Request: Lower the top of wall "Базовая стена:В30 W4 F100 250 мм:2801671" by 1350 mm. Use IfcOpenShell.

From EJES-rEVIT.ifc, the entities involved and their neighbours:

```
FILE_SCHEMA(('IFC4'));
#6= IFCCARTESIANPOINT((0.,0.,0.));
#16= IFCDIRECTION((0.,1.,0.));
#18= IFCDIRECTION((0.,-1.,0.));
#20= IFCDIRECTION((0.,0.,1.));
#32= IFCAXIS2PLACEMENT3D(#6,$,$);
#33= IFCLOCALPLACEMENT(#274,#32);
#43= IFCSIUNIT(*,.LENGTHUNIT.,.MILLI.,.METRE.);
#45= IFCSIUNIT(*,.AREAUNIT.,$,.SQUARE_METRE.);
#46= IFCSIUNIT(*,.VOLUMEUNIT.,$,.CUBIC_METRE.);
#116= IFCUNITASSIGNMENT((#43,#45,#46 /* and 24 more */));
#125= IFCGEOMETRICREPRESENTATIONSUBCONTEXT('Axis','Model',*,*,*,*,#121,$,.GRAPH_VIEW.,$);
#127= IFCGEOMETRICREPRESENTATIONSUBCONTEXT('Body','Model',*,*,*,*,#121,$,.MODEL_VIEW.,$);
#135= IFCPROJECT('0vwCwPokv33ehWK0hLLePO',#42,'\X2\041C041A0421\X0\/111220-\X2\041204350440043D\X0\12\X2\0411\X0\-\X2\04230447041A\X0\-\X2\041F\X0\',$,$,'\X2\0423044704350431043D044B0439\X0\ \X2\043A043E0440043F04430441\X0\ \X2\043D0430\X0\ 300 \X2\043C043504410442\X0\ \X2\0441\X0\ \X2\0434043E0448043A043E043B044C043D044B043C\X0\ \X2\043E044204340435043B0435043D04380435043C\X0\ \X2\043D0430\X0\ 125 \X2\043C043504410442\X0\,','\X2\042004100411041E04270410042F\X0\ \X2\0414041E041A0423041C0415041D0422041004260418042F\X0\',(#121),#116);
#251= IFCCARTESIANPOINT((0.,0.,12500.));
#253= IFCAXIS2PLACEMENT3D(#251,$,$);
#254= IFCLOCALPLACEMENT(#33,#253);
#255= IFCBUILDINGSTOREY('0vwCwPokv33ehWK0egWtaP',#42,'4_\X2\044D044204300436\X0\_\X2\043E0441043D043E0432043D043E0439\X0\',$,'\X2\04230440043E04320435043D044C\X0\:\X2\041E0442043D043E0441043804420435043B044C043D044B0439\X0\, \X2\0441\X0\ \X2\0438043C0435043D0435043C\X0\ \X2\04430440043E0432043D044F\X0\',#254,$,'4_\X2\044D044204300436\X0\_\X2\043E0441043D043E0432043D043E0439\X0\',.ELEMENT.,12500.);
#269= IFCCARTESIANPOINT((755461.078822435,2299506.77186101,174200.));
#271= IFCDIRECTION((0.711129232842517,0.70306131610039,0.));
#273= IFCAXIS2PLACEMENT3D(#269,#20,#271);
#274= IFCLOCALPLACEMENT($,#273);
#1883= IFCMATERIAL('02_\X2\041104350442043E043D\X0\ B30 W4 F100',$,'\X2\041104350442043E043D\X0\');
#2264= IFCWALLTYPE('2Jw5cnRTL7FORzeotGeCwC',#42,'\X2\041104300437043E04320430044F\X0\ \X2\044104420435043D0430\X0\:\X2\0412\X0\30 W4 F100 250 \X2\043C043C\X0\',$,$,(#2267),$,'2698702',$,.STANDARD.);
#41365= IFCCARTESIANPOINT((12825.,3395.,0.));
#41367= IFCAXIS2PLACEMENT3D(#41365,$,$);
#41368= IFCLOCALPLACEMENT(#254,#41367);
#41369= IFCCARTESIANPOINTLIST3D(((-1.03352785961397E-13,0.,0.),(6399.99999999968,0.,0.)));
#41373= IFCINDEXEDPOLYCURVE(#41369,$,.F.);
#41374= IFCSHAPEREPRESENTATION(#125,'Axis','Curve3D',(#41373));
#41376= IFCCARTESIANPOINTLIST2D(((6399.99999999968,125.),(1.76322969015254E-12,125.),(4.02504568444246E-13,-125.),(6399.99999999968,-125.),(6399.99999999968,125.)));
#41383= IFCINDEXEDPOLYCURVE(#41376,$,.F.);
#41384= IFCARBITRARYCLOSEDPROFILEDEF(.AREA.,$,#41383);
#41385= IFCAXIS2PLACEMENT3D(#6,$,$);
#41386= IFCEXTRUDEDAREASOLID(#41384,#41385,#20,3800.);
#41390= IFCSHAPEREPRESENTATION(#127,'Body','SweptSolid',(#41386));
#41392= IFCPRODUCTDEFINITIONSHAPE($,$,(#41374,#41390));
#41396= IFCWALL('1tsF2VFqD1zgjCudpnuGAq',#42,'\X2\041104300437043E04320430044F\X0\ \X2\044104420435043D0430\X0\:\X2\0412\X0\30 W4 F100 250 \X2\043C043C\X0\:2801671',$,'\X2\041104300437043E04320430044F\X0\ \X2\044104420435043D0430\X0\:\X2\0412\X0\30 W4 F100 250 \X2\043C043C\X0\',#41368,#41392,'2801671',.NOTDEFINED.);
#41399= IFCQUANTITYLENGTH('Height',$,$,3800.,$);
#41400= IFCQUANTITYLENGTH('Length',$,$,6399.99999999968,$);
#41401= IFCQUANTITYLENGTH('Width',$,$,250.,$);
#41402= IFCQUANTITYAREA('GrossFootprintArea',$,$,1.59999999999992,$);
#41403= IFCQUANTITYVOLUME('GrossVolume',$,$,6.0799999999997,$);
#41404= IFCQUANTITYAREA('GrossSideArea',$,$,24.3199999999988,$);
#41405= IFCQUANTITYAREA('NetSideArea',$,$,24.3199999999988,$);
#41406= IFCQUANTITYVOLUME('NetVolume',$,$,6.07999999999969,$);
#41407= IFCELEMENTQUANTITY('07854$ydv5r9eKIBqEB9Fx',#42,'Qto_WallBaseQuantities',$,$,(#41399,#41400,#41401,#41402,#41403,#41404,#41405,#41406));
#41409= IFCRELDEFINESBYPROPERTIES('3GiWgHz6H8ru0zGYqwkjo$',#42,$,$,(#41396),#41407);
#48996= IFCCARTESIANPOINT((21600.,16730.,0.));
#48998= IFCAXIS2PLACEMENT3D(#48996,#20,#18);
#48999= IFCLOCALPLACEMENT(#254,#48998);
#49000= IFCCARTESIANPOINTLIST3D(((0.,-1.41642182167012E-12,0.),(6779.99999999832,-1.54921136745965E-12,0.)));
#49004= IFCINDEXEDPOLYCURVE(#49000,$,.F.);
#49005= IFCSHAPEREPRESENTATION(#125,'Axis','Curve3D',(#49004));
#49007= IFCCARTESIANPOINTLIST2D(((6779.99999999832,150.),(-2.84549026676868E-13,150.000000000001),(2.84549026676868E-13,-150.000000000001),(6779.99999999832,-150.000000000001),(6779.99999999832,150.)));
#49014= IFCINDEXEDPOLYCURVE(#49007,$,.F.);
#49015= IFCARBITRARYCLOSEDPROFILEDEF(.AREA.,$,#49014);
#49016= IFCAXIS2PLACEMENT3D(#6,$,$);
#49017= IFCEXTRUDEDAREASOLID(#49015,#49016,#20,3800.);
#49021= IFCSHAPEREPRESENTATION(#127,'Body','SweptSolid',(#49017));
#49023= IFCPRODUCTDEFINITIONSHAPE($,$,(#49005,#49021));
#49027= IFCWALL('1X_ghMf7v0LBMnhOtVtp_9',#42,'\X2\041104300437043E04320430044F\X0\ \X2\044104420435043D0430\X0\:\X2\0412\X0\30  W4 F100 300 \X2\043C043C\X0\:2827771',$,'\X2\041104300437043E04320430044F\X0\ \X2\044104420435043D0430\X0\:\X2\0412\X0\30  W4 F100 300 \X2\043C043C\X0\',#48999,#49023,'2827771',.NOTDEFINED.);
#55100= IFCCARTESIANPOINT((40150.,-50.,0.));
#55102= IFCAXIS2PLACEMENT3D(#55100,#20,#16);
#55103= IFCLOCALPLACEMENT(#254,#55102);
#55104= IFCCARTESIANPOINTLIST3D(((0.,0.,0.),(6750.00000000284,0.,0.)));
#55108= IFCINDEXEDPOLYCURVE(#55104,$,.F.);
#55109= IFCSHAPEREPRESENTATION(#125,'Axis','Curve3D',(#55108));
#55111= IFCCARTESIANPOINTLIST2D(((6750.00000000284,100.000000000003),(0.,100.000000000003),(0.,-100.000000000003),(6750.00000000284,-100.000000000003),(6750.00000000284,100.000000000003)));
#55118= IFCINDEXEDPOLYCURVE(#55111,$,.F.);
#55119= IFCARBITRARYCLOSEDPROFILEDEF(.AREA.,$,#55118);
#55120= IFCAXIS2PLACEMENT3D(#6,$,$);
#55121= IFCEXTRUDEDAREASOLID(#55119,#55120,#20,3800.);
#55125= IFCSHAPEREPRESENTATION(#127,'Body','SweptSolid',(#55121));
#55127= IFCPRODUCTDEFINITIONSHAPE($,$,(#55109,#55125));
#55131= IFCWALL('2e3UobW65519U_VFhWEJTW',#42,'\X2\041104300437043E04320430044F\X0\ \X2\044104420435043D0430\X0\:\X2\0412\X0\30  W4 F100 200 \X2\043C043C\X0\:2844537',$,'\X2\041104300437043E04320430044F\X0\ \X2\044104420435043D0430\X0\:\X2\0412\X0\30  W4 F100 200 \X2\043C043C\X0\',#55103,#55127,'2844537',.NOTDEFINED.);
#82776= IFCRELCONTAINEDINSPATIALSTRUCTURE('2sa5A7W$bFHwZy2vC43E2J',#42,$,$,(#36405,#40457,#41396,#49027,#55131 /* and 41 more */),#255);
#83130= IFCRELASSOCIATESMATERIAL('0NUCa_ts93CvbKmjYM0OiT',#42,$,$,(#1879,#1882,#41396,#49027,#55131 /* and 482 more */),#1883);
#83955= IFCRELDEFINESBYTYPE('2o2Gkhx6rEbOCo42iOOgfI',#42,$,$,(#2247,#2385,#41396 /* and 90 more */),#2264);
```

```python
import ifcopenshell
import ifcopenshell.api.pset
import ifcopenshell.geom
import ifcopenshell.util.element
import ifcopenshell.util.representation
import ifcopenshell.util.shape
import ifcopenshell.util.unit

model = ifcopenshell.open("EJES-rEVIT.ifc")
unit_scale = ifcopenshell.util.unit.calculate_unit_scale(model)
area_scale = ifcopenshell.util.unit.calculate_unit_scale(model, "AREAUNIT")
volume_scale = ifcopenshell.util.unit.calculate_unit_scale(model, "VOLUMEUNIT")
settings = ifcopenshell.geom.settings()


def volume(element):
    """Net volume in cubic metres, openings subtracted."""
    shape = ifcopenshell.geom.create_shape(settings, element)
    return ifcopenshell.util.shape.get_volume(shape.geometry)


wall = model.by_id(41396)
before = volume(wall)

body = ifcopenshell.util.representation.get_representation(wall, "Model", "Body")
solid = body.Items[0]
old_height = solid.Depth
solid.Depth -= 1350.0
after = volume(wall)
thickness = 0.25  # wall thickness in metres

# Update the stored height, areas and volumes.
qto = model.by_id(ifcopenshell.util.element.get_pset(wall, "Qto_WallBaseQuantities", should_inherit=False)["id"])
ifcopenshell.api.pset.edit_qto(model, qto=qto, properties={
    "Height": solid.Depth,
    "GrossVolume": ifcopenshell.util.element.get_pset(wall, "Qto_WallBaseQuantities", "GrossVolume") * solid.Depth / old_height,
    "GrossSideArea": ifcopenshell.util.element.get_pset(wall, "Qto_WallBaseQuantities", "GrossSideArea") * solid.Depth / old_height,
    "NetSideArea": after / thickness / area_scale,
    "NetVolume": after / volume_scale,
})

print(f"height {old_height:g} -> {solid.Depth:g}, volume {before:.3f} -> {after:.3f} m3")

model.write("EJES-rEVIT-out.ifc")
```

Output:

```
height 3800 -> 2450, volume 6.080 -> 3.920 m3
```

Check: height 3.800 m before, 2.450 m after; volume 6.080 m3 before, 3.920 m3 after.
